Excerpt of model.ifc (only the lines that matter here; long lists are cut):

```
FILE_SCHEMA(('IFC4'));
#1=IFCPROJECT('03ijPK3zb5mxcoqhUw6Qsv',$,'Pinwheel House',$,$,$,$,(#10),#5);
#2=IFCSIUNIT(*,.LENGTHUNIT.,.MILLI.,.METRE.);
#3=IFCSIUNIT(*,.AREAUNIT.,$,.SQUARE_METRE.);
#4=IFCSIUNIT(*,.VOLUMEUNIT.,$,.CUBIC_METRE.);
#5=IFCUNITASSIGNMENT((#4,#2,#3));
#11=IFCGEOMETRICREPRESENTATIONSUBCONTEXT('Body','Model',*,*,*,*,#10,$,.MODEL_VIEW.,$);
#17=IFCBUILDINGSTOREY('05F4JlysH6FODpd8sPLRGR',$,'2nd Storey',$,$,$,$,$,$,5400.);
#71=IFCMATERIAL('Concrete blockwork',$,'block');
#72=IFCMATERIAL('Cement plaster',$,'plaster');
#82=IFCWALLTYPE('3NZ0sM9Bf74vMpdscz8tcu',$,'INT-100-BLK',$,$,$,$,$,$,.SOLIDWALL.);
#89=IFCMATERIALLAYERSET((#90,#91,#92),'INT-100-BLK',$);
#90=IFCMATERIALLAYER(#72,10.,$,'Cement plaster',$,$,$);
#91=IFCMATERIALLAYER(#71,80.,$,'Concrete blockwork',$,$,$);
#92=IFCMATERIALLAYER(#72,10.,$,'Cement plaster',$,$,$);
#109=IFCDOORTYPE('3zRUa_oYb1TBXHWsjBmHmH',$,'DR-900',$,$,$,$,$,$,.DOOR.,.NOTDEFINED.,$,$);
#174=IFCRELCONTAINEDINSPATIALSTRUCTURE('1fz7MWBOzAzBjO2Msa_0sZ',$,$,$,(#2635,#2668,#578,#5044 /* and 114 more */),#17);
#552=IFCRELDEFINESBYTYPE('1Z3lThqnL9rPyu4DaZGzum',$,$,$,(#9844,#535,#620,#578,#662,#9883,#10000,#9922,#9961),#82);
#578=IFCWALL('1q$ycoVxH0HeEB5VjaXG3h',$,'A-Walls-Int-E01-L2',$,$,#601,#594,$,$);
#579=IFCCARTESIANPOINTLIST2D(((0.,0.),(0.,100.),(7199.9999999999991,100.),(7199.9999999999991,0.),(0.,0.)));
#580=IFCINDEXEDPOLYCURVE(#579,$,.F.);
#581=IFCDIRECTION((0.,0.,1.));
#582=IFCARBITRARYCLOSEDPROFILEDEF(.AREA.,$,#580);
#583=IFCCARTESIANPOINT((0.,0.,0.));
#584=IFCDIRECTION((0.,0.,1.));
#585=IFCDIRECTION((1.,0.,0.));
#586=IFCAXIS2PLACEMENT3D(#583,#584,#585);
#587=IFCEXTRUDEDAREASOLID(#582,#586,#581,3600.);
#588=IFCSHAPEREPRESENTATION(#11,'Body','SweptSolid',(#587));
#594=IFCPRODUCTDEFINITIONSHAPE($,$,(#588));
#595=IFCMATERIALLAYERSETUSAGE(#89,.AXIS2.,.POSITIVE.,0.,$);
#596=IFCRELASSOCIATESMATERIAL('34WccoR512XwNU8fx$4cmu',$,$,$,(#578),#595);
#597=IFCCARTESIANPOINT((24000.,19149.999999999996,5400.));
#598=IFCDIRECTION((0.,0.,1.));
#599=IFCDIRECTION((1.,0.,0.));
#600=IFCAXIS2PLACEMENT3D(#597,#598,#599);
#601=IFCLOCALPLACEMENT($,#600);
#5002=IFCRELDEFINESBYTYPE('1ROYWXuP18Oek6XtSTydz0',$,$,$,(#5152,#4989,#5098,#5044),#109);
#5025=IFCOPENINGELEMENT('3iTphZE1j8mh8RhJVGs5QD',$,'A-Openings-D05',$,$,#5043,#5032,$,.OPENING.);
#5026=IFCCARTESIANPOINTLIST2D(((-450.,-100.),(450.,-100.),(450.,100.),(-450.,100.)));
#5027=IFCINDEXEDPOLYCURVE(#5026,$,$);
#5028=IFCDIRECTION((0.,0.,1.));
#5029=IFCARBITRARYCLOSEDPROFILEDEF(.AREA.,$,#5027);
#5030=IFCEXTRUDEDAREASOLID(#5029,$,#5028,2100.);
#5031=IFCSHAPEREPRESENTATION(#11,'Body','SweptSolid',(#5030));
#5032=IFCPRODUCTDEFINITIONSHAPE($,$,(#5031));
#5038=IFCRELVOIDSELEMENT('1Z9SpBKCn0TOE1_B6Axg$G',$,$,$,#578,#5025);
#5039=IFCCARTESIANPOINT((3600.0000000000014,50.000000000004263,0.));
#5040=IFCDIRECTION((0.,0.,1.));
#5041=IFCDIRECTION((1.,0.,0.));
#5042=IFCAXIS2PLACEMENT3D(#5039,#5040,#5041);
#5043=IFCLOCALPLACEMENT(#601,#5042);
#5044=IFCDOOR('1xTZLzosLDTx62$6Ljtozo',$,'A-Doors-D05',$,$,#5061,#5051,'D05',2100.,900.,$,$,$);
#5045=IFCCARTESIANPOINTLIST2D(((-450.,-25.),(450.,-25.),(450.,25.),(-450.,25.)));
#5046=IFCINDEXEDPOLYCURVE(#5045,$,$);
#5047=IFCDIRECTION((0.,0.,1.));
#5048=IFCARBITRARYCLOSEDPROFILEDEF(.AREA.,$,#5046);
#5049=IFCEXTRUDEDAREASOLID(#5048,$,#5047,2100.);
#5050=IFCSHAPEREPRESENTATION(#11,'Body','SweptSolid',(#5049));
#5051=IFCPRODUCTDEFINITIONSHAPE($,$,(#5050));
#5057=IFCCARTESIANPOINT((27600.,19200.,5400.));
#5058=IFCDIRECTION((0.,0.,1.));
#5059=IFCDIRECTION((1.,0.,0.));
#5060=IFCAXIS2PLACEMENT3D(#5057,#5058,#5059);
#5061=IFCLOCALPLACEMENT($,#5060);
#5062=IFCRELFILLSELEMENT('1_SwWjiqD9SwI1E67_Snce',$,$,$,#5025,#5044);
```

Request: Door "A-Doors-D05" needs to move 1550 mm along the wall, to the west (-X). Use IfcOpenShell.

```python
import ifcopenshell
import ifcopenshell.api.geometry
import ifcopenshell.util.placement

model = ifcopenshell.open("model.ifc")

door = model.by_guid("1xTZLzosLDTx62$6Ljtozo")
opening = door.FillsVoids[0].RelatingOpeningElement
wall = opening.VoidsElements[0].RelatingBuildingElement

wall_matrix = ifcopenshell.util.placement.get_local_placement(wall.ObjectPlacement)
shift = wall_matrix[:3, 0] * -1550.0
before = ifcopenshell.util.placement.get_local_placement(door.ObjectPlacement)[:3, 3].copy()

# The door is not placed relative to its opening, so move both.
for product in (opening, door):
    matrix = ifcopenshell.util.placement.get_local_placement(product.ObjectPlacement)
    matrix[:3, 3] += shift
    ifcopenshell.api.geometry.edit_object_placement(model, product=product, matrix=matrix, is_si=False)

after = ifcopenshell.util.placement.get_local_placement(door.ObjectPlacement)[:3, 3]
print("door moved by", (after - before).round(3) + 0.0)

model.write("model_updated.ifc")
```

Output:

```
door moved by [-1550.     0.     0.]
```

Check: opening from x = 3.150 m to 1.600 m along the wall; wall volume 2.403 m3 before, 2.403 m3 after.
